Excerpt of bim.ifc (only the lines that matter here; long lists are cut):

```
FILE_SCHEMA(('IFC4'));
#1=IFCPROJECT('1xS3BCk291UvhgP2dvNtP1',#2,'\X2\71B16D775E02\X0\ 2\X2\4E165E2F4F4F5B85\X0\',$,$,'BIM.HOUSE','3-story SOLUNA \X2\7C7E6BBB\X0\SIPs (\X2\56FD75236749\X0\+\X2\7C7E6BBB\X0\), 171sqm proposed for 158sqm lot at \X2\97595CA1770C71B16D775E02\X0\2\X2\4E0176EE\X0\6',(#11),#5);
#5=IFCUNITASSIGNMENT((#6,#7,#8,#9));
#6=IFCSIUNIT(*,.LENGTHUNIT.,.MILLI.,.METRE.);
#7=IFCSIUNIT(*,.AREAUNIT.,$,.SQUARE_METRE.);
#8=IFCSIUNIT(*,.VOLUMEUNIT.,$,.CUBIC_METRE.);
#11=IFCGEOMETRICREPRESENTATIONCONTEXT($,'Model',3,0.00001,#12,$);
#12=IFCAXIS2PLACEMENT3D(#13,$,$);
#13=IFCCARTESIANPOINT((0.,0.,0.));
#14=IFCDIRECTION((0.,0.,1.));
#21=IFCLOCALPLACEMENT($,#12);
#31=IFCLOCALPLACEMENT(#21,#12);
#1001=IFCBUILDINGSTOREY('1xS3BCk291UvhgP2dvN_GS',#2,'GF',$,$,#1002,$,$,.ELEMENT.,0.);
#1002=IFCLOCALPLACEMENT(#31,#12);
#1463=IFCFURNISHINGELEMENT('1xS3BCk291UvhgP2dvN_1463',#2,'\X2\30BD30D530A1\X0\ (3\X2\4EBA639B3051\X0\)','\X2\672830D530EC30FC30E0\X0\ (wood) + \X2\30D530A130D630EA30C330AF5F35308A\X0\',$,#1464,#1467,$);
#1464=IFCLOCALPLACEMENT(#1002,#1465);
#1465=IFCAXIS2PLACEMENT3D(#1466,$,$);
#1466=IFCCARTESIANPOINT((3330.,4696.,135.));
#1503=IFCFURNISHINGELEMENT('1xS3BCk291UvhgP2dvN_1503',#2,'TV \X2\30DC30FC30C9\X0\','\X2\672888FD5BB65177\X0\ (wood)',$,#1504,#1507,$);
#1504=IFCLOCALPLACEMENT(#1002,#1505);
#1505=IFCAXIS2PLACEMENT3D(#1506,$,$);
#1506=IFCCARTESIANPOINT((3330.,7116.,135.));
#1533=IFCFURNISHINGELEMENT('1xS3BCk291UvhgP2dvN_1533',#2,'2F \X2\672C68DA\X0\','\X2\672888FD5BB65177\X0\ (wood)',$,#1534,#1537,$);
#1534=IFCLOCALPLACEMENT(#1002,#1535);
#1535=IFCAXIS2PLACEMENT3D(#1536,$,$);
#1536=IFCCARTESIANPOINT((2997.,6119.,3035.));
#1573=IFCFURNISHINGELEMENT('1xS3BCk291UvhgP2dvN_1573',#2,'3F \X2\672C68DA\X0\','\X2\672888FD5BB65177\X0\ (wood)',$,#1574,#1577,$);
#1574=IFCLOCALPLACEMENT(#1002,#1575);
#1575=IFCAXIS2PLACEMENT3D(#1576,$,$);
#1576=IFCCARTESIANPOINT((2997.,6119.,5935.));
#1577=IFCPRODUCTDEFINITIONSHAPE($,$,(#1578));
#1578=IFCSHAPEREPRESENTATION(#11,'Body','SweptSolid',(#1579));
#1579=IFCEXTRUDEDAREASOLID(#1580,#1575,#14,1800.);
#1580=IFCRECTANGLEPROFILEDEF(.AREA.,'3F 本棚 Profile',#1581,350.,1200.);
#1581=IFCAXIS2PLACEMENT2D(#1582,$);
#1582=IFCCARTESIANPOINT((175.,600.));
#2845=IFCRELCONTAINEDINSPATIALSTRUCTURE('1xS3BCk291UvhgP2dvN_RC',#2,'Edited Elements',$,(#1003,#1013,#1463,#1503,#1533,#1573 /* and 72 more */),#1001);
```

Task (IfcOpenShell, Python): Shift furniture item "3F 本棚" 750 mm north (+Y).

```python
import ifcopenshell
import ifcopenshell.api.geometry
import ifcopenshell.util.placement

model = ifcopenshell.open("bim.ifc")

item = model.by_guid("1xS3BCk291UvhgP2dvN_1573")
matrix = ifcopenshell.util.placement.get_local_placement(item.ObjectPlacement)
matrix[1, 3] += 750.0
ifcopenshell.api.geometry.edit_object_placement(model, product=item, matrix=matrix, is_si=False)

print(ifcopenshell.util.placement.get_local_placement(item.ObjectPlacement).round(3) + 0.0)

model.write("bim_v2.ifc")
```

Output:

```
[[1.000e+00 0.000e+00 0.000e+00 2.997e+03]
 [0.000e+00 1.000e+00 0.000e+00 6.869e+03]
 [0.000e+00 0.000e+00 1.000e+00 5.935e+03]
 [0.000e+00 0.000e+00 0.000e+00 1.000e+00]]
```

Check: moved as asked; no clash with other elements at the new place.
